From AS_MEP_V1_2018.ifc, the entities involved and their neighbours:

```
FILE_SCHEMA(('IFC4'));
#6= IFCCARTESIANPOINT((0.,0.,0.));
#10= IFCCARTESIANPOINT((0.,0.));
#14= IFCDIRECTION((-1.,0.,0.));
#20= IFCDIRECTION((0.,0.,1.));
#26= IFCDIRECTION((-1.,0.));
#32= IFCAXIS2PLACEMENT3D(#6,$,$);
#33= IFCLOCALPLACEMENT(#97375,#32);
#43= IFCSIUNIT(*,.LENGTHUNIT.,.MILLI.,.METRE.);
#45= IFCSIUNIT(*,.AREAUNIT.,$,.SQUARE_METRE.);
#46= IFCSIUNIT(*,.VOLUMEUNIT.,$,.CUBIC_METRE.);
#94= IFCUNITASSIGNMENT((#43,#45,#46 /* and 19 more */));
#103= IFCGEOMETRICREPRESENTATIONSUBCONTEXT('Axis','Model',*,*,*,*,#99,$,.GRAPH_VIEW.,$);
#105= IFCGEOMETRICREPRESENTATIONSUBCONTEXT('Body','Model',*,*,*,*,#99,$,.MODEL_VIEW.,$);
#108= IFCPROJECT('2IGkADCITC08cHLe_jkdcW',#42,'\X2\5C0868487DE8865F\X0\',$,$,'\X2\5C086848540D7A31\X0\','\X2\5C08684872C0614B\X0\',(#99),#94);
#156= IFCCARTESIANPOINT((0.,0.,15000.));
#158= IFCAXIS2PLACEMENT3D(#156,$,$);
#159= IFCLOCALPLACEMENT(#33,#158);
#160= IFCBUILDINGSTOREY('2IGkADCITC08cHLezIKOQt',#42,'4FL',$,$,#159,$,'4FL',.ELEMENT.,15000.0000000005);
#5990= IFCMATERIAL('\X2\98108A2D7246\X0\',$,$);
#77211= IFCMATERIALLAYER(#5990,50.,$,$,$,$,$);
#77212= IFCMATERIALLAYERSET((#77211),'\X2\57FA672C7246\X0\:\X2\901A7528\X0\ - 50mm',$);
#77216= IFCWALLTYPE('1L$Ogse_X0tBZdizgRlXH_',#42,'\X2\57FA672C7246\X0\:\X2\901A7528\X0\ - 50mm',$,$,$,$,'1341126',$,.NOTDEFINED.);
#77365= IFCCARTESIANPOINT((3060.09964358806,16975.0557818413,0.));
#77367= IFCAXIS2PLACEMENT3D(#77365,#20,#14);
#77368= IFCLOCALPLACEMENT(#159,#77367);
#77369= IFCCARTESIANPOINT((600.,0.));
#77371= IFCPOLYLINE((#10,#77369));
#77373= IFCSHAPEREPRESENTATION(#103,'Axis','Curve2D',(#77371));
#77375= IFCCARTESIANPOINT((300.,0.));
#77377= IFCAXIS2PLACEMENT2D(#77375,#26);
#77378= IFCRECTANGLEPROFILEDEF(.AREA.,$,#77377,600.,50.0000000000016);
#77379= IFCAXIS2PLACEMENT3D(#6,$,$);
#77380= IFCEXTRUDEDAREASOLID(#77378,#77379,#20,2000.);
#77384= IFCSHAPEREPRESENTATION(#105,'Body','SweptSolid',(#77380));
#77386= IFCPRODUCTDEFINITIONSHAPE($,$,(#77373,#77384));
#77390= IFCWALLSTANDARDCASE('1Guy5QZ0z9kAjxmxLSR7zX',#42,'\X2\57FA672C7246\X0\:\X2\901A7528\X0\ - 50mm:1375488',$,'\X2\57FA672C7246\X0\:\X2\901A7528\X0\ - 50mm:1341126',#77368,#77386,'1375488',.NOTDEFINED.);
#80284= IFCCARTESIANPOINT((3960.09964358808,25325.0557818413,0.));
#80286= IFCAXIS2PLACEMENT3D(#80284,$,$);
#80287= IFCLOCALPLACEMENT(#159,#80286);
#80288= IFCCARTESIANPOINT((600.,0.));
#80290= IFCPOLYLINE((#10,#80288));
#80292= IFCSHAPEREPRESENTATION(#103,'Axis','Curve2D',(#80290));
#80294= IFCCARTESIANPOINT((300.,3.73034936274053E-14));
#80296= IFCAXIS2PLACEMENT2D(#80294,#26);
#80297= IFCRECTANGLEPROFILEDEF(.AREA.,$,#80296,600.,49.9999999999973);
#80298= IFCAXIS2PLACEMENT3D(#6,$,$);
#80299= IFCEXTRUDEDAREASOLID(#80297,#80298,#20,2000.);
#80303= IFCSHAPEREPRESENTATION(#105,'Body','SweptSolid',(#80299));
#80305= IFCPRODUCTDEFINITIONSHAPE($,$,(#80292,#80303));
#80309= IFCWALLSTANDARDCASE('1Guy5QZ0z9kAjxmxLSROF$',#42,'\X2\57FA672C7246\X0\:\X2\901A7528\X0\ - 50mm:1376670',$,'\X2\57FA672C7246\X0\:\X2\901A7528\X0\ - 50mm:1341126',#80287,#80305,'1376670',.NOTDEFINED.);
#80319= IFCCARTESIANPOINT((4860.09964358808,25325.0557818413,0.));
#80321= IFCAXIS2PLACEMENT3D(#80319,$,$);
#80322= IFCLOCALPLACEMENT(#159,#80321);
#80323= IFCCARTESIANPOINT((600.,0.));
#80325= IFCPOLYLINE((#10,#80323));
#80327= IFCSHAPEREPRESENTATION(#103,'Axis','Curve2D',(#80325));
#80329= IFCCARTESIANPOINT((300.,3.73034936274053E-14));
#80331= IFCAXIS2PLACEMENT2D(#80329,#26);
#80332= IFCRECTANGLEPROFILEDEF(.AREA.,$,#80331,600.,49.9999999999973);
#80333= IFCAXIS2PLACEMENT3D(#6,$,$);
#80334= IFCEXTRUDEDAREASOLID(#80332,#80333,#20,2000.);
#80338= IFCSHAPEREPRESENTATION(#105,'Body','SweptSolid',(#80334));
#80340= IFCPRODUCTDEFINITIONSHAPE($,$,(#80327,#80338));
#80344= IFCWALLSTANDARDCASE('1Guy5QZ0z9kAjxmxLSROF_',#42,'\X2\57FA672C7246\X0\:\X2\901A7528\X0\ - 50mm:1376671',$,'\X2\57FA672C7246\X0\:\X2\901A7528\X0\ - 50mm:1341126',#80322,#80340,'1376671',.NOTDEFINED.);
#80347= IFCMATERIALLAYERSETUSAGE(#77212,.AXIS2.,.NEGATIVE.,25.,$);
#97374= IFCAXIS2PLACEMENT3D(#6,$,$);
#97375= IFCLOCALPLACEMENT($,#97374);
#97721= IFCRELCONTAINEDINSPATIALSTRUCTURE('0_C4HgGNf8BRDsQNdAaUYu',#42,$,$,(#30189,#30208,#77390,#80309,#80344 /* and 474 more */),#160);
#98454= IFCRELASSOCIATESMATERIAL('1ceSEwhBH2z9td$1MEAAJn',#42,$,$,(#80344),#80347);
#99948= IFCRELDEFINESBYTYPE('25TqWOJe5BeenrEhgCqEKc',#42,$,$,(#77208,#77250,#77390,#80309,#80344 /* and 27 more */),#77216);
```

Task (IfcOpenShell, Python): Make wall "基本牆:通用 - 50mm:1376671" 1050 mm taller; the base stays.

```python
import ifcopenshell
import ifcopenshell.geom
import ifcopenshell.util.representation
import ifcopenshell.util.shape

model = ifcopenshell.open("AS_MEP_V1_2018.ifc")
settings = ifcopenshell.geom.settings()


def volume(element):
    """Net volume in cubic metres, openings subtracted."""
    shape = ifcopenshell.geom.create_shape(settings, element)
    return ifcopenshell.util.shape.get_volume(shape.geometry)


wall = model.by_guid("1Guy5QZ0z9kAjxmxLSROF_")
before = volume(wall)

body = ifcopenshell.util.representation.get_representation(wall, "Model", "Body")
solid = body.Items[0]
old_height = solid.Depth
solid.Depth += 1050.0
after = volume(wall)

print(f"height {old_height:g} -> {solid.Depth:g}, volume {before:.3f} -> {after:.3f} m3")

model.write("AS_MEP_V1_2018_v2.ifc")
```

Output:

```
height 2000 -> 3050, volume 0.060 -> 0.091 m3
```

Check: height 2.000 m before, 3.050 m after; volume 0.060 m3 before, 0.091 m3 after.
